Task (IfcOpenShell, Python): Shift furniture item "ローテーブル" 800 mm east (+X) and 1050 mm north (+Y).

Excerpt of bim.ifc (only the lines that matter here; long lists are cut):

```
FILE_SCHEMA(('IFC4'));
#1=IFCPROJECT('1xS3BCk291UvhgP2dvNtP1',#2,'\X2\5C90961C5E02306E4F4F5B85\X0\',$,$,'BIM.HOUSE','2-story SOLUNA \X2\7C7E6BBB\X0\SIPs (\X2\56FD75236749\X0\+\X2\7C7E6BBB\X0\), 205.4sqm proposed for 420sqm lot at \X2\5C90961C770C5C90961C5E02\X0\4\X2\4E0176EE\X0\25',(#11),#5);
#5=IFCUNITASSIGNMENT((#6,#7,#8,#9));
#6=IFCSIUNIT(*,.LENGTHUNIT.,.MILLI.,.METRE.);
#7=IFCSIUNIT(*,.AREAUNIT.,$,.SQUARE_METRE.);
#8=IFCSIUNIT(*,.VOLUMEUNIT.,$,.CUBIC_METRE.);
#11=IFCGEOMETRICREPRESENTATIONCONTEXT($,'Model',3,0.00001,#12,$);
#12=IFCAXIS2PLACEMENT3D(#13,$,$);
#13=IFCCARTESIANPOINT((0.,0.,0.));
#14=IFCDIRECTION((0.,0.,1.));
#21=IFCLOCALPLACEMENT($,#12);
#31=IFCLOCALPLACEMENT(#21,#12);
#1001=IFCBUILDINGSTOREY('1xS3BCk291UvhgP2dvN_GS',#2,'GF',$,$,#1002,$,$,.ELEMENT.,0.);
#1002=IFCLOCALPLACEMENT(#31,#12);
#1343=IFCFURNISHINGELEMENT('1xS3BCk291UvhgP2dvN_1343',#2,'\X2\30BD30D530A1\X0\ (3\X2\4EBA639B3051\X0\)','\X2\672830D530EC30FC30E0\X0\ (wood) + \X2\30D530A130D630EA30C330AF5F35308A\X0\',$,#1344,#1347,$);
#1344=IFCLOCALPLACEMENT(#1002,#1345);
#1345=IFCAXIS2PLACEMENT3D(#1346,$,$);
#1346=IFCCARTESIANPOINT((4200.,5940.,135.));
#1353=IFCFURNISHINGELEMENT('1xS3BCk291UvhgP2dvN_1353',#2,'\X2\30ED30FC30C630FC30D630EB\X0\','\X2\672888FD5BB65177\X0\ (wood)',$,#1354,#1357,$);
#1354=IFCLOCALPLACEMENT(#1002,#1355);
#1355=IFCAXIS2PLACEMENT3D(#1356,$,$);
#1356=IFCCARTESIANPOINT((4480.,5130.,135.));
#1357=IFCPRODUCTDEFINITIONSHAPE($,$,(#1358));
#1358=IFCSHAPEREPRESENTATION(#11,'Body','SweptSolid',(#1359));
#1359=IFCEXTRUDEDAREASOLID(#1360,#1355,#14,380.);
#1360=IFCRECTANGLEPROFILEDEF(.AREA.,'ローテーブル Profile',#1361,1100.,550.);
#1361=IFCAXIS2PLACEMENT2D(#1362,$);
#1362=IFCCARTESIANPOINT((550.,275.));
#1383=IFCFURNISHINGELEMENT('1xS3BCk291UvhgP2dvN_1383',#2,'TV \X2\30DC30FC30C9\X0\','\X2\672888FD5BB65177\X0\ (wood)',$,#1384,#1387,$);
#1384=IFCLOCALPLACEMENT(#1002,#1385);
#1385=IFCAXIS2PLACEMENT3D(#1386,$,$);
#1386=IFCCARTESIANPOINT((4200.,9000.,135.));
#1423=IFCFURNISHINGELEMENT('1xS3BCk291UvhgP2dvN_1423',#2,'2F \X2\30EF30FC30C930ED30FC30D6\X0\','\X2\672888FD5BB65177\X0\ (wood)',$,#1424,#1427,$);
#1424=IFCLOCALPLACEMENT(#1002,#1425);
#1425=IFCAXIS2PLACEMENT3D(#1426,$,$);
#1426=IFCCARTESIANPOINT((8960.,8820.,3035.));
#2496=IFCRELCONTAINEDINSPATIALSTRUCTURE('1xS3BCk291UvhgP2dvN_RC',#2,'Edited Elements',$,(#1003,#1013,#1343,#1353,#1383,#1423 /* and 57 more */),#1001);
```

```python
import ifcopenshell
import ifcopenshell.api.geometry
import ifcopenshell.util.placement
import ifcopenshell.util.unit

model = ifcopenshell.open("bim.ifc")
unit_scale = ifcopenshell.util.unit.calculate_unit_scale(model)

item = model.by_guid("1xS3BCk291UvhgP2dvN_1353")
matrix = ifcopenshell.util.placement.get_local_placement(item.ObjectPlacement)
matrix[0, 3] += 0.8 / unit_scale
matrix[1, 3] += 1.05 / unit_scale
ifcopenshell.api.geometry.edit_object_placement(model, product=item, matrix=matrix, is_si=False)

print(ifcopenshell.util.placement.get_local_placement(item.ObjectPlacement).round(3) + 0.0)

model.write("bim_rev.ifc")
```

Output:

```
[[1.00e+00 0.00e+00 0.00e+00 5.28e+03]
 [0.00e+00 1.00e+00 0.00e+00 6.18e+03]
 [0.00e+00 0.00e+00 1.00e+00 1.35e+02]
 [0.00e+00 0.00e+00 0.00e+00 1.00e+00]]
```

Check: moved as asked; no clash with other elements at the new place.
